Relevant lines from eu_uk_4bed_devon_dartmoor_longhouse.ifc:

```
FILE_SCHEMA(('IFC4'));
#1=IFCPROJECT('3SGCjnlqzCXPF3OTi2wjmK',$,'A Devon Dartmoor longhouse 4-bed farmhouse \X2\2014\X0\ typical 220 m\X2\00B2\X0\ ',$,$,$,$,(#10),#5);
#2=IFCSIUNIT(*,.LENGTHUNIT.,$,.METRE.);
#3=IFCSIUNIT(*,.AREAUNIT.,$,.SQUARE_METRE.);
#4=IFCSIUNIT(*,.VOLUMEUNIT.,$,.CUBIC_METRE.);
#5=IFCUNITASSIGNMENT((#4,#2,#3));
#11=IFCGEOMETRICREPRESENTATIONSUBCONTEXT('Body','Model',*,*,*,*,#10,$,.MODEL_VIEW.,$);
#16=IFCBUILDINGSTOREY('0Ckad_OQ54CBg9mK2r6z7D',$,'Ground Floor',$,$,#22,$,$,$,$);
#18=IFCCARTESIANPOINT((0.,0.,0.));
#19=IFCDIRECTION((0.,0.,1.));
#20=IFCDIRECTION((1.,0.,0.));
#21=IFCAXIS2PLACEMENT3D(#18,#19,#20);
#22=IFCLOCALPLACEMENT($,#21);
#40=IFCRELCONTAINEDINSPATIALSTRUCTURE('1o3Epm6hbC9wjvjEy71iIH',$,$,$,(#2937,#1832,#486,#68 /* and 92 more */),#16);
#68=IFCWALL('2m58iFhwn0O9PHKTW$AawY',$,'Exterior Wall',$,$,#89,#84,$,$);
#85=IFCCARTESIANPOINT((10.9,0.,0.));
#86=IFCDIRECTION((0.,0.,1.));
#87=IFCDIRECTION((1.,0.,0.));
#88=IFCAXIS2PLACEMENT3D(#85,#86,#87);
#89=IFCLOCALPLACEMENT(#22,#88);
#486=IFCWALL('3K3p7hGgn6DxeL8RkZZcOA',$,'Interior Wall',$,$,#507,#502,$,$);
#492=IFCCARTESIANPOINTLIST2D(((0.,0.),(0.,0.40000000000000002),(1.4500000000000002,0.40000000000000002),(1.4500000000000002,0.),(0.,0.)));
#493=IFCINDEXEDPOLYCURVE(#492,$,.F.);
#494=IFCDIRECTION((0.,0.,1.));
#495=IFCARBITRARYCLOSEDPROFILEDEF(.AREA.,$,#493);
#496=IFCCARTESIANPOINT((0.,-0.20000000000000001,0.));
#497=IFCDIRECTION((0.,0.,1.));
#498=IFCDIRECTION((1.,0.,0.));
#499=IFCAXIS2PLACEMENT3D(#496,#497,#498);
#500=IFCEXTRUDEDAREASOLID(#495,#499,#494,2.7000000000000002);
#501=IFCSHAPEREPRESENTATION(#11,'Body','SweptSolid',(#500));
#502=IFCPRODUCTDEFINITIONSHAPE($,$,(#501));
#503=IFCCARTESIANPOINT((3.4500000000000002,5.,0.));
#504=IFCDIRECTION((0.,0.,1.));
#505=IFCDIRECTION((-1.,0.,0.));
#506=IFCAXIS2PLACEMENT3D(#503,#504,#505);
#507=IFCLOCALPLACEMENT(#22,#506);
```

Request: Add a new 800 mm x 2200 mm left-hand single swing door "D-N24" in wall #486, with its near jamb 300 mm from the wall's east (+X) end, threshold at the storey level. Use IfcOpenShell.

```python
import numpy as np
import ifcopenshell
import ifcopenshell.api.feature
import ifcopenshell.api.geometry
import ifcopenshell.api.root
import ifcopenshell.api.spatial
import ifcopenshell.geom
import ifcopenshell.util.element
import ifcopenshell.util.placement
import ifcopenshell.util.representation
import ifcopenshell.util.shape
import ifcopenshell.util.unit

model = ifcopenshell.open("eu_uk_4bed_devon_dartmoor_longhouse.ifc")
unit_scale = ifcopenshell.util.unit.calculate_unit_scale(model)
settings = ifcopenshell.geom.settings()


def volume(element):
    """Net volume in cubic metres, openings subtracted."""
    shape = ifcopenshell.geom.create_shape(settings, element)
    return ifcopenshell.util.shape.get_volume(shape.geometry)


wall = model.by_guid("3K3p7hGgn6DxeL8RkZZcOA")
storey = ifcopenshell.util.element.get_container(wall, ifc_class="IfcBuildingStorey")
context = ifcopenshell.util.representation.get_context(model, "Model", "Body", "MODEL_VIEW")
before = volume(wall)

width, height, from_end, sill = 0.8, 2.2, 0.3, 0.0  # metres

# The wall runs along its own X axis, and the end named is its -X end.
wall_shape = ifcopenshell.geom.create_shape(settings, wall)
x, y, z = ifcopenshell.util.shape.get_vertices(wall_shape.geometry).T
start = x.min() + from_end
face, thickness = float(y.min()), float(y.max() - y.min())
wall_matrix = ifcopenshell.util.placement.get_local_placement(wall.ObjectPlacement)
level = ifcopenshell.util.placement.get_local_placement(storey.ObjectPlacement)[2, 3]


def in_wall(x, y):
    """Placement at x, y metres in the wall's axes, at sill height."""
    matrix = wall_matrix.copy()
    matrix[:, 3] = wall_matrix @ np.array([x / unit_scale, y / unit_scale, 0.0, 1.0])
    matrix[2, 3] = level + sill / unit_scale
    return matrix


# Opening: a box that overshoots both wall faces by 50 mm.
opening = ifcopenshell.api.root.create_entity(model, ifc_class="IfcOpeningElement", predefined_type="OPENING")
box = ifcopenshell.api.geometry.add_wall_representation(
    model, context=context, length=width, height=height, thickness=thickness + 0.1
)
ifcopenshell.api.geometry.assign_representation(model, product=opening, representation=box)
ifcopenshell.api.geometry.edit_object_placement(model, product=opening, matrix=in_wall(start, face - 0.05), is_si=False)
ifcopenshell.api.feature.add_feature(model, feature=opening, element=wall)

door = ifcopenshell.api.root.create_entity(model, ifc_class="IfcDoor", name="D-N24", predefined_type="DOOR")
door.OverallWidth, door.OverallHeight = width / unit_scale, height / unit_scale
door.OperationType = "SINGLE_SWING_LEFT"
body = ifcopenshell.api.geometry.add_door_representation(
    model,
    context=context,
    overall_width=door.OverallWidth,
    overall_height=door.OverallHeight,
    operation_type="SINGLE_SWING_LEFT",
    lining_properties={"LiningDepth": thickness / unit_scale, "ThresholdDepth": thickness / unit_scale},
)
ifcopenshell.api.geometry.assign_representation(model, product=door, representation=body)
ifcopenshell.api.spatial.assign_container(model, products=[door], relating_structure=storey)
ifcopenshell.api.feature.add_filling(model, opening=opening, element=door)

# The lining spans the wall, so the door starts at the wall face.
ifcopenshell.api.geometry.edit_object_placement(model, product=door, matrix=in_wall(start, face), is_si=False)

after = volume(wall)

print(f"wall volume {before:.3f} -> {after:.3f} m3")

model.write("eu_uk_4bed_devon_dartmoor_longhouse_rev.ifc")
```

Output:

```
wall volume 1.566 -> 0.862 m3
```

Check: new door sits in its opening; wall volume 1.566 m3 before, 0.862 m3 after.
